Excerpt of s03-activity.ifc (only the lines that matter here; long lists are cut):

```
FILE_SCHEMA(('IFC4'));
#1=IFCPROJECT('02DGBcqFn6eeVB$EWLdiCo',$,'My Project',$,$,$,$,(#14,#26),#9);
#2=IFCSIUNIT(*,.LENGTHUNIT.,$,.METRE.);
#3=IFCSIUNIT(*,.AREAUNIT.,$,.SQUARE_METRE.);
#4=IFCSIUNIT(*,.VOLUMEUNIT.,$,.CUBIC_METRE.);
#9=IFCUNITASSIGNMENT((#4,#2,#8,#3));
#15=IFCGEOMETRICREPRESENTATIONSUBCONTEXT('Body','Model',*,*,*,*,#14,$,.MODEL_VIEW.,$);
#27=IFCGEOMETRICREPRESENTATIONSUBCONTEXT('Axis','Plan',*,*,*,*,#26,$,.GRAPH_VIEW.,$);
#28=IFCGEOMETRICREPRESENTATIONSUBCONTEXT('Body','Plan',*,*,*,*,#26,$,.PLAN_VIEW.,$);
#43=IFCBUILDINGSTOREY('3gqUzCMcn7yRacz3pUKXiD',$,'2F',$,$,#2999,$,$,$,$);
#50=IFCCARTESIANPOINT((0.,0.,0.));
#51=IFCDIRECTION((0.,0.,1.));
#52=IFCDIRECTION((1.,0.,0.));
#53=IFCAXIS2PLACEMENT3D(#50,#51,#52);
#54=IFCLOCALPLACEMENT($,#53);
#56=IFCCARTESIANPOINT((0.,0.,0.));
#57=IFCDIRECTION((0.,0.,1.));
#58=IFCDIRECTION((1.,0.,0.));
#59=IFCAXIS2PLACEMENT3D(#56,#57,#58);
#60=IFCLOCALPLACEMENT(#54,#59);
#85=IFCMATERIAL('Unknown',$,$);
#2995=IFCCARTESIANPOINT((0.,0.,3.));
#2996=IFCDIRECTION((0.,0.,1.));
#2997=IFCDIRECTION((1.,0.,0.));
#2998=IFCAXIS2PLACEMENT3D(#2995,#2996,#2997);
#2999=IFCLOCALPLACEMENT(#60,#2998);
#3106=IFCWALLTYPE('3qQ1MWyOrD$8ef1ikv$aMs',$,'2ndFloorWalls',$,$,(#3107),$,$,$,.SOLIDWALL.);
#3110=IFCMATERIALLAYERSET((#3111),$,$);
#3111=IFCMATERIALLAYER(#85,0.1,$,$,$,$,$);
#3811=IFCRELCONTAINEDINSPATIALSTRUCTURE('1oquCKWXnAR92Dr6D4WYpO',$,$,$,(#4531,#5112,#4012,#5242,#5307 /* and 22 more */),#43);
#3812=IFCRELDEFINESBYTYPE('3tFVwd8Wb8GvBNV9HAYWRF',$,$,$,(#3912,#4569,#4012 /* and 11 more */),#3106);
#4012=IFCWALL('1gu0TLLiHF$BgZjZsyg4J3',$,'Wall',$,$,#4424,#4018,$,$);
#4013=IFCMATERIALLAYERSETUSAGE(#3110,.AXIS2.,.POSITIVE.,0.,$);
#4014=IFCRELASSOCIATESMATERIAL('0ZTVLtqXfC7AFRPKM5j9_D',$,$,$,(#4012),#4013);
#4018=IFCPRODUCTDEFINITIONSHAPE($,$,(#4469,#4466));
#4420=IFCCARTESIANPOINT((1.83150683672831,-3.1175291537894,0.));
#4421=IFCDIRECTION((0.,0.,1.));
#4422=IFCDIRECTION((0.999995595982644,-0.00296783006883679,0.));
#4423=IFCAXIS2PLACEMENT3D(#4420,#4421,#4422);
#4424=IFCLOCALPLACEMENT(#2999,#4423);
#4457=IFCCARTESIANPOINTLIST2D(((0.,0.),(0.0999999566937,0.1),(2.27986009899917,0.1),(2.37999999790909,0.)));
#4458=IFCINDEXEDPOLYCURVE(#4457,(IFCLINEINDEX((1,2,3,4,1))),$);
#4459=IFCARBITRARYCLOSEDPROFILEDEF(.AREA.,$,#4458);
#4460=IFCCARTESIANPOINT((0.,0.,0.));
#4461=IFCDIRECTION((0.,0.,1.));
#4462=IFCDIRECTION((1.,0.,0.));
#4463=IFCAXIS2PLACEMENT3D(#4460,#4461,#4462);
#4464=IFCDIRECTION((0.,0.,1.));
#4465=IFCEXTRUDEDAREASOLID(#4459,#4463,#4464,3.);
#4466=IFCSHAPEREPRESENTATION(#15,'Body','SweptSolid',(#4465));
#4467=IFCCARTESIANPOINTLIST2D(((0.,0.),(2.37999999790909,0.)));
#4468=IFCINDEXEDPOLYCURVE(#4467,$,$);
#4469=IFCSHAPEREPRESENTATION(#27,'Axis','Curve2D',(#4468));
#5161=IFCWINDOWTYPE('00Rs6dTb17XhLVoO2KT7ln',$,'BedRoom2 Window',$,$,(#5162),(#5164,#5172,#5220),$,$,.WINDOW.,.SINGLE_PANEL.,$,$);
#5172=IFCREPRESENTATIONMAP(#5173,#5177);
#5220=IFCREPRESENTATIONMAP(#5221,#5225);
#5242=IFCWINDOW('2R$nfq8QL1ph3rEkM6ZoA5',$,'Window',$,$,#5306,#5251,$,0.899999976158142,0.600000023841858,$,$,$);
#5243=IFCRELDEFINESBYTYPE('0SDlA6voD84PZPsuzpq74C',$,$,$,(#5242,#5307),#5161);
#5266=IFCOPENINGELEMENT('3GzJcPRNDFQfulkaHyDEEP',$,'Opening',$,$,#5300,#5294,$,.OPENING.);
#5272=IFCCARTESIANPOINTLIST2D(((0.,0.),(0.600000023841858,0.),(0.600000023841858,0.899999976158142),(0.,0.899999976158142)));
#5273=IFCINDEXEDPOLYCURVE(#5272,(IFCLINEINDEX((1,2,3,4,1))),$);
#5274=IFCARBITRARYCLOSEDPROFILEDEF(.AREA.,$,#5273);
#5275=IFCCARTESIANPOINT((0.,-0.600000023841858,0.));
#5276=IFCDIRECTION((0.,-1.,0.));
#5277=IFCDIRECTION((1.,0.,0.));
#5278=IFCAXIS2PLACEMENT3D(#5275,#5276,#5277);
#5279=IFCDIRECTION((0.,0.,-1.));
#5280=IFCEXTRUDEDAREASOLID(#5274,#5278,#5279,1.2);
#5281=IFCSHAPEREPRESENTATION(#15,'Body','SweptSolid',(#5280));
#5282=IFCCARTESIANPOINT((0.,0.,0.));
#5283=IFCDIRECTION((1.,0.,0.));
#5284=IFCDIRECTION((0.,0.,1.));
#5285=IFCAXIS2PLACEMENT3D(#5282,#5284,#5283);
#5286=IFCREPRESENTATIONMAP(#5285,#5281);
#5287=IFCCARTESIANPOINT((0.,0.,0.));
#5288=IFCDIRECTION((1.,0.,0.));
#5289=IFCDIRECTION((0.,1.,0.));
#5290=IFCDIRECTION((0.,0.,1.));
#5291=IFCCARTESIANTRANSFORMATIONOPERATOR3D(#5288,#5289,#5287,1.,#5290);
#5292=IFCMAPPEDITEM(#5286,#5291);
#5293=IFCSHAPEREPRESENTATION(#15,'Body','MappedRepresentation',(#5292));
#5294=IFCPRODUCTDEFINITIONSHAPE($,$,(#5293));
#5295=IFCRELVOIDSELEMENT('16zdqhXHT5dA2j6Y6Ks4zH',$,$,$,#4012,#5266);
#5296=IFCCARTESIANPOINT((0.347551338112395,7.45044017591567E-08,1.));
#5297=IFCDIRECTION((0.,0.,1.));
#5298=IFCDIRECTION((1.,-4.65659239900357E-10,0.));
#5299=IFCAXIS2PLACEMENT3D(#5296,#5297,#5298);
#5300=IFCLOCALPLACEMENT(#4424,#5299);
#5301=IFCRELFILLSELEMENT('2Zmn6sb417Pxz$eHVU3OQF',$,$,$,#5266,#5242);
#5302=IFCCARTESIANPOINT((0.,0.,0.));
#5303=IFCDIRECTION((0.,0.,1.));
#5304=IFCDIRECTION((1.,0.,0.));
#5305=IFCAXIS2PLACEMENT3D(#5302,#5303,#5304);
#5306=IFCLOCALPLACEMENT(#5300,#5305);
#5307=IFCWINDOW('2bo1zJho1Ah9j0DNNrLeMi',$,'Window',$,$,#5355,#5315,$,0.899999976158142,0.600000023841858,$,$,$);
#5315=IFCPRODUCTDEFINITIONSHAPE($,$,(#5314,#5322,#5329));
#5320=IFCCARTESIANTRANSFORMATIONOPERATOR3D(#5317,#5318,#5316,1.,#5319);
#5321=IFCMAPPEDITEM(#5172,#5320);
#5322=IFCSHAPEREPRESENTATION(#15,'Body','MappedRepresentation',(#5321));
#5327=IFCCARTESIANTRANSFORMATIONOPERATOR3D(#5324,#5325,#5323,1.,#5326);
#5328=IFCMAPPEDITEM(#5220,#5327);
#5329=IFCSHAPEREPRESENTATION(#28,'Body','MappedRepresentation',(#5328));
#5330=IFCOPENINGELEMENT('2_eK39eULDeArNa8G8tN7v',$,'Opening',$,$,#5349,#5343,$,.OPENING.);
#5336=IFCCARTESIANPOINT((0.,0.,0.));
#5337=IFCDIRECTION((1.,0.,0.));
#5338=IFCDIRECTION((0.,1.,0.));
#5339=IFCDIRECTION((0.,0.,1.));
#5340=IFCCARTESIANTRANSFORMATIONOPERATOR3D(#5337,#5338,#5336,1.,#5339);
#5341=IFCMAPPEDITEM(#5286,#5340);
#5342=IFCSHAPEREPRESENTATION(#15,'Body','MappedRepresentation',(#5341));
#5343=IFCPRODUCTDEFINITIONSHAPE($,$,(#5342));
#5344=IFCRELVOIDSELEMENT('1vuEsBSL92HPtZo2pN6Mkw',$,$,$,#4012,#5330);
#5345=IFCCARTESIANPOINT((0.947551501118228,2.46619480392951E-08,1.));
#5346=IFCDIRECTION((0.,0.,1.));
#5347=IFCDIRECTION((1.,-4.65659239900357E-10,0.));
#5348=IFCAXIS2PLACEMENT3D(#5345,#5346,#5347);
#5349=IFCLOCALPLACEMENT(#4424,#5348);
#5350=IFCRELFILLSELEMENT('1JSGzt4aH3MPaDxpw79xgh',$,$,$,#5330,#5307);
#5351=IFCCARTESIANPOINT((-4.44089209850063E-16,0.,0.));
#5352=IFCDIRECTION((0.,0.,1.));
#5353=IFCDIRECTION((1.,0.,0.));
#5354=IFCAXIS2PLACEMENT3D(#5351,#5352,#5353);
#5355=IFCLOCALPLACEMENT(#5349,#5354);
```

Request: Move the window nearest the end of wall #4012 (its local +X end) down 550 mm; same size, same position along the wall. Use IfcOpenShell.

```python
import numpy as np
import ifcopenshell
import ifcopenshell.api.geometry
import ifcopenshell.util.placement
import ifcopenshell.util.unit

model = ifcopenshell.open("s03-activity.ifc")
unit_scale = ifcopenshell.util.unit.calculate_unit_scale(model)

window = model.by_guid("2bo1zJho1Ah9j0DNNrLeMi")
opening = window.FillsVoids[0].RelatingOpeningElement
dz = -0.55

shift = np.array([0.0, 0.0, dz])
# The window is placed relative to its opening, so it follows when the opening moves.
matrix = ifcopenshell.util.placement.get_local_placement(opening.ObjectPlacement)
matrix[:3, 3] += shift
ifcopenshell.api.geometry.edit_object_placement(
    model, product=opening, matrix=matrix, is_si=False, should_transform_children=True
)

print(f"moved by {dz * unit_scale:+.3f} m")

model.write("s03-activity_v2.ifc")
```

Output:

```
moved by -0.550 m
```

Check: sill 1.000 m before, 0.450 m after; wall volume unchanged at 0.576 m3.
